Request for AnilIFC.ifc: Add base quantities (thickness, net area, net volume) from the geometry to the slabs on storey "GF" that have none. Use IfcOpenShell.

First a look at what the model holds.

```python
import ifcopenshell
import ifcopenshell.util.element
import ifcopenshell.util.unit

model = ifcopenshell.open("AnilIFC.ifc")
print(model.schema)
for unit_type in ("LENGTHUNIT", "AREAUNIT", "VOLUMEUNIT"):
    print(unit_type, ifcopenshell.util.unit.calculate_unit_scale(model, unit_type))
storey = next(s for s in model.by_type("IfcBuildingStorey") if s.Name == "GF")
slabs = [e for e in ifcopenshell.util.element.get_decomposition(storey) if e.is_a("IfcSlab")]
for e in sorted(slabs, key=lambda e: e.id()):
    print(e.id(), e.is_a(), e.Name, list(ifcopenshell.util.element.get_psets(e, qtos_only=True)), sep=" | ")
```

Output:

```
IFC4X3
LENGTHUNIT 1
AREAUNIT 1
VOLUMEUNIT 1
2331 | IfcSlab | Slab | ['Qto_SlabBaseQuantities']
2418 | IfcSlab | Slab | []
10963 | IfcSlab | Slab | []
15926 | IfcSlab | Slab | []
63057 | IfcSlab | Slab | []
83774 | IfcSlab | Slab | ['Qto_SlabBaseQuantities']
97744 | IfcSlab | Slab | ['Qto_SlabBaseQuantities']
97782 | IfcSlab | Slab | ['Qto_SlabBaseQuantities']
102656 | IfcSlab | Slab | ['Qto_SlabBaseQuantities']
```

```python
import ifcopenshell
import ifcopenshell.api.pset
import ifcopenshell.geom
import ifcopenshell.util.element
import ifcopenshell.util.shape
import ifcopenshell.util.unit

model = ifcopenshell.open("AnilIFC.ifc")
unit_scale = ifcopenshell.util.unit.calculate_unit_scale(model)
area_scale = ifcopenshell.util.unit.calculate_unit_scale(model, "AREAUNIT")
volume_scale = ifcopenshell.util.unit.calculate_unit_scale(model, "VOLUMEUNIT")
settings = ifcopenshell.geom.settings()

storey = next(s for s in model.by_type("IfcBuildingStorey") if s.Name == "GF")
slabs = [e for e in ifcopenshell.util.element.get_decomposition(storey) if e.is_a("IfcSlab")]

for e in sorted(slabs, key=lambda e: e.id()):
    if ifcopenshell.util.element.get_psets(e, qtos_only=True, should_inherit=False):
        continue
    # Geometry comes back in metres, in the element's own axes.
    shape = ifcopenshell.geom.create_shape(settings, e)
    values = {
        "Width": ifcopenshell.util.shape.get_z(shape.geometry) / unit_scale,
        "NetArea": ifcopenshell.util.shape.get_footprint_area(shape.geometry) / area_scale,
        "NetVolume": ifcopenshell.util.shape.get_volume(shape.geometry) / volume_scale,
    }
    qto = ifcopenshell.api.pset.add_qto(model, product=e, name="Qto_SlabBaseQuantities")
    ifcopenshell.api.pset.edit_qto(model, qto=qto, properties=values)
    print(e.id(), {k: round(v, 3) for k, v in values.items()})

model.write("AnilIFC_updated.ifc")
```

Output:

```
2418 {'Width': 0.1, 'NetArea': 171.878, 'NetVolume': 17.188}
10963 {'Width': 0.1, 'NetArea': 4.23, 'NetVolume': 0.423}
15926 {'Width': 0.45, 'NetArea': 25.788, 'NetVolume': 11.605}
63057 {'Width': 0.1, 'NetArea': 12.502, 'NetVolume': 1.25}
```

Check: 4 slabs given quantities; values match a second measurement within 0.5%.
